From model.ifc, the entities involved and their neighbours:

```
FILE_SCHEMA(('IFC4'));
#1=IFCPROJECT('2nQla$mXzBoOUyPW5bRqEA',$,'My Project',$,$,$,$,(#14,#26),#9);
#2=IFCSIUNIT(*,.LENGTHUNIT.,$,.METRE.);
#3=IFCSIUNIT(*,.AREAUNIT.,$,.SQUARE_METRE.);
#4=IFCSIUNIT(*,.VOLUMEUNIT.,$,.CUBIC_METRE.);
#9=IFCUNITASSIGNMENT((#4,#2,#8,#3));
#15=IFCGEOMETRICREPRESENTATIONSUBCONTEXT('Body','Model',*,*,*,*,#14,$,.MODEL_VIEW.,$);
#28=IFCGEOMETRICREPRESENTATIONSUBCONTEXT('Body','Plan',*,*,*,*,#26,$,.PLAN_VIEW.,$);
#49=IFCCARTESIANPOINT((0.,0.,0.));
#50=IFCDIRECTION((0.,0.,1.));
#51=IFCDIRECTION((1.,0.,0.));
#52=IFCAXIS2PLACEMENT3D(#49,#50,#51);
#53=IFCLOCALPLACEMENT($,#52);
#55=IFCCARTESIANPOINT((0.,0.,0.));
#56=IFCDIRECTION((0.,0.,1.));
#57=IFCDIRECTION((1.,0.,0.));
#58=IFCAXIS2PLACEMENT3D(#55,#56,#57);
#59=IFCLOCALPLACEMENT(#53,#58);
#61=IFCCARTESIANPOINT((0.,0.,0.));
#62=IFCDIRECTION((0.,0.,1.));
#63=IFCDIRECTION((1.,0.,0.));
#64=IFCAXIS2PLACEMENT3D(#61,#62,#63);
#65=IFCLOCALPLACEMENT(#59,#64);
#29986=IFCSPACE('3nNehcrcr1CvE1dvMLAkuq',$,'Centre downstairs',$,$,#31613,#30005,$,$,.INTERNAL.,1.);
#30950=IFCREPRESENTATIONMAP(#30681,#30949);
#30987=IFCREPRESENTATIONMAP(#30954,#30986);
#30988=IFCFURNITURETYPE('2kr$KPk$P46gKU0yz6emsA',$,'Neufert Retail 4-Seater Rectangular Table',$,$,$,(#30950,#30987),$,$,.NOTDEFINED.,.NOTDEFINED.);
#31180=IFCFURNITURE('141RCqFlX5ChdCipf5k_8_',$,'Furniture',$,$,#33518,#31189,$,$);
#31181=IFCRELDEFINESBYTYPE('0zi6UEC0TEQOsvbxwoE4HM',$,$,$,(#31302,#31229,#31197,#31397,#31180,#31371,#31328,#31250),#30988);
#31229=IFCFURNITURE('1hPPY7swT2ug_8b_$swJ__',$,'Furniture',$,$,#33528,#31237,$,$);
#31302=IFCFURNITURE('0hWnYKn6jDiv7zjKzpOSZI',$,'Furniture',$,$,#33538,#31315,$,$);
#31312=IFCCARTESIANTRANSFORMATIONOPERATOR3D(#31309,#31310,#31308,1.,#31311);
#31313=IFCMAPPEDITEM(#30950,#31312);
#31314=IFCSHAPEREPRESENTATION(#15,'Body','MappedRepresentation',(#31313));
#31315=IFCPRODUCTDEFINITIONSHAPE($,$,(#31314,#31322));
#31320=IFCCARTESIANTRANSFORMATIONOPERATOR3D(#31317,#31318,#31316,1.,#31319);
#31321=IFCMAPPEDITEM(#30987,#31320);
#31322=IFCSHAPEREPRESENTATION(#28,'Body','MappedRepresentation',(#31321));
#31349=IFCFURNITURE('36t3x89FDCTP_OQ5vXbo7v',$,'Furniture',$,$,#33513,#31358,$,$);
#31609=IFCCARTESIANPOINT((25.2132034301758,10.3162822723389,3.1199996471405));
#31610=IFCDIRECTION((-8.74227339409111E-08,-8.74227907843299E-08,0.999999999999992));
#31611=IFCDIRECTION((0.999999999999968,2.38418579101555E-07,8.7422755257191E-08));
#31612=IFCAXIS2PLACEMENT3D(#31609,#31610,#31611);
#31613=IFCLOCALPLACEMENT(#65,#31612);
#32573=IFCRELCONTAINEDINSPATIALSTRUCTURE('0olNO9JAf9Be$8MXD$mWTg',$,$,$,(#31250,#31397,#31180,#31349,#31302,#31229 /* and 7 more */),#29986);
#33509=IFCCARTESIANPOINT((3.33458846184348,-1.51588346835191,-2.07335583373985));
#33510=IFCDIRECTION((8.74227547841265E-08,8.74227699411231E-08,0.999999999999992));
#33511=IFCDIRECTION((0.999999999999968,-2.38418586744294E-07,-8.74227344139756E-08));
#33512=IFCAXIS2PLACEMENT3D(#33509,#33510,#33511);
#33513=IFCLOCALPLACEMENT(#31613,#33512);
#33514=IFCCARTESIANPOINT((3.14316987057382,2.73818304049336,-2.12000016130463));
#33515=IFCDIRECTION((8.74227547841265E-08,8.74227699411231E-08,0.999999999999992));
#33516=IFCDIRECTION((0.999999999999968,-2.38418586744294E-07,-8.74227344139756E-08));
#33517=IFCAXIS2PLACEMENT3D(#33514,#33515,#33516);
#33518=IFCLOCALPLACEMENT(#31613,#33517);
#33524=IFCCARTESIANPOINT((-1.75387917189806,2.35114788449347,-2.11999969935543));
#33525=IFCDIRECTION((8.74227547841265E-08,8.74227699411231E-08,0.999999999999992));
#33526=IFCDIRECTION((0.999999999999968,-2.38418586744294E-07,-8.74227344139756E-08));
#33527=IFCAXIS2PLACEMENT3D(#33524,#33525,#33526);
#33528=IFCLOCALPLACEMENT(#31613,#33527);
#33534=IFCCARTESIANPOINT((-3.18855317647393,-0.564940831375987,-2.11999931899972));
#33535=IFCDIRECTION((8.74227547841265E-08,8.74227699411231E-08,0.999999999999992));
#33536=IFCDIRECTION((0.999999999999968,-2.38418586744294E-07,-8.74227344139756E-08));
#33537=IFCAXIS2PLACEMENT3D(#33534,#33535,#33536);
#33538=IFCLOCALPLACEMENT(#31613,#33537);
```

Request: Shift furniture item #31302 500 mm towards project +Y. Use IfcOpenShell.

```python
import ifcopenshell
import ifcopenshell.api.geometry
import ifcopenshell.util.placement
import ifcopenshell.util.unit

model = ifcopenshell.open("model.ifc")
unit_scale = ifcopenshell.util.unit.calculate_unit_scale(model)

item = model.by_guid("0hWnYKn6jDiv7zjKzpOSZI")
matrix = ifcopenshell.util.placement.get_local_placement(item.ObjectPlacement)
matrix[1, 3] += 0.5 / unit_scale
ifcopenshell.api.geometry.edit_object_placement(model, product=item, matrix=matrix, is_si=False)

print(ifcopenshell.util.placement.get_local_placement(item.ObjectPlacement).round(3) + 0.0)

model.write("model_edited.ifc")
```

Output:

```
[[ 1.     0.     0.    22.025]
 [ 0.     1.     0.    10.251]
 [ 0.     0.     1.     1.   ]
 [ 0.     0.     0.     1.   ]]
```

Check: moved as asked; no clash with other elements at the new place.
